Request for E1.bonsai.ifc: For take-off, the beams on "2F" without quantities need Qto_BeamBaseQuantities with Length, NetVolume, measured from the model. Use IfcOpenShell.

First a look at what the model holds.

```python
import ifcopenshell
import ifcopenshell.util.element
import ifcopenshell.util.unit

model = ifcopenshell.open("E1.bonsai.ifc")
print(model.schema)
for unit_type in ("LENGTHUNIT", "AREAUNIT", "VOLUMEUNIT"):
    print(unit_type, ifcopenshell.util.unit.calculate_unit_scale(model, unit_type))
storey = next(s for s in model.by_type("IfcBuildingStorey") if s.Name == "2F")
beams = [e for e in ifcopenshell.util.element.get_decomposition(storey) if e.is_a("IfcBeam")]
for e in sorted(beams, key=lambda e: e.id()):
    print(e.id(), e.is_a(), e.Name, list(ifcopenshell.util.element.get_psets(e, qtos_only=True)), sep=" | ")
```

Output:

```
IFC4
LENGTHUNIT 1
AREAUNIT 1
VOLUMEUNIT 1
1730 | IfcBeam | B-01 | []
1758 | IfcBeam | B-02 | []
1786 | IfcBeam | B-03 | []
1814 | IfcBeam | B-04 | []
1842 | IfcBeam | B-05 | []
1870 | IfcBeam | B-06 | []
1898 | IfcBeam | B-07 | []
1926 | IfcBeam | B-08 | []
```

```python
import ifcopenshell
import ifcopenshell.api.pset
import ifcopenshell.geom
import ifcopenshell.util.element
import ifcopenshell.util.shape
import ifcopenshell.util.unit

model = ifcopenshell.open("E1.bonsai.ifc")
unit_scale = ifcopenshell.util.unit.calculate_unit_scale(model)
volume_scale = ifcopenshell.util.unit.calculate_unit_scale(model, "VOLUMEUNIT")
settings = ifcopenshell.geom.settings()

storey = next(s for s in model.by_type("IfcBuildingStorey") if s.Name == "2F")
beams = [e for e in ifcopenshell.util.element.get_decomposition(storey) if e.is_a("IfcBeam")]

for e in sorted(beams, key=lambda e: e.id()):
    if ifcopenshell.util.element.get_psets(e, qtos_only=True, should_inherit=False):
        continue
    # Geometry comes back in metres, in the element's own axes.
    shape = ifcopenshell.geom.create_shape(settings, e)
    values = {
        "Length": ifcopenshell.util.shape.get_max_xyz(shape.geometry) / unit_scale,
        "NetVolume": ifcopenshell.util.shape.get_volume(shape.geometry) / volume_scale,
    }
    qto = ifcopenshell.api.pset.add_qto(model, product=e, name="Qto_BeamBaseQuantities")
    ifcopenshell.api.pset.edit_qto(model, qto=qto, properties=values)
    print(e.id(), {k: round(v, 3) for k, v in values.items()})

model.write("E1.bonsai_rev.ifc")
```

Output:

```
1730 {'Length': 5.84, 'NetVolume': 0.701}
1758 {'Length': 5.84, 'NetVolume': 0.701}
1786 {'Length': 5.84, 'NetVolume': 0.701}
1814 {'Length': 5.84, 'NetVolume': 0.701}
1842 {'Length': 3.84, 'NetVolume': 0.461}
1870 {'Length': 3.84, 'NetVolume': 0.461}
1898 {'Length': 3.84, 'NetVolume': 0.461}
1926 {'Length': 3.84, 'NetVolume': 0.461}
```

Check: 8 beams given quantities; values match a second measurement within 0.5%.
